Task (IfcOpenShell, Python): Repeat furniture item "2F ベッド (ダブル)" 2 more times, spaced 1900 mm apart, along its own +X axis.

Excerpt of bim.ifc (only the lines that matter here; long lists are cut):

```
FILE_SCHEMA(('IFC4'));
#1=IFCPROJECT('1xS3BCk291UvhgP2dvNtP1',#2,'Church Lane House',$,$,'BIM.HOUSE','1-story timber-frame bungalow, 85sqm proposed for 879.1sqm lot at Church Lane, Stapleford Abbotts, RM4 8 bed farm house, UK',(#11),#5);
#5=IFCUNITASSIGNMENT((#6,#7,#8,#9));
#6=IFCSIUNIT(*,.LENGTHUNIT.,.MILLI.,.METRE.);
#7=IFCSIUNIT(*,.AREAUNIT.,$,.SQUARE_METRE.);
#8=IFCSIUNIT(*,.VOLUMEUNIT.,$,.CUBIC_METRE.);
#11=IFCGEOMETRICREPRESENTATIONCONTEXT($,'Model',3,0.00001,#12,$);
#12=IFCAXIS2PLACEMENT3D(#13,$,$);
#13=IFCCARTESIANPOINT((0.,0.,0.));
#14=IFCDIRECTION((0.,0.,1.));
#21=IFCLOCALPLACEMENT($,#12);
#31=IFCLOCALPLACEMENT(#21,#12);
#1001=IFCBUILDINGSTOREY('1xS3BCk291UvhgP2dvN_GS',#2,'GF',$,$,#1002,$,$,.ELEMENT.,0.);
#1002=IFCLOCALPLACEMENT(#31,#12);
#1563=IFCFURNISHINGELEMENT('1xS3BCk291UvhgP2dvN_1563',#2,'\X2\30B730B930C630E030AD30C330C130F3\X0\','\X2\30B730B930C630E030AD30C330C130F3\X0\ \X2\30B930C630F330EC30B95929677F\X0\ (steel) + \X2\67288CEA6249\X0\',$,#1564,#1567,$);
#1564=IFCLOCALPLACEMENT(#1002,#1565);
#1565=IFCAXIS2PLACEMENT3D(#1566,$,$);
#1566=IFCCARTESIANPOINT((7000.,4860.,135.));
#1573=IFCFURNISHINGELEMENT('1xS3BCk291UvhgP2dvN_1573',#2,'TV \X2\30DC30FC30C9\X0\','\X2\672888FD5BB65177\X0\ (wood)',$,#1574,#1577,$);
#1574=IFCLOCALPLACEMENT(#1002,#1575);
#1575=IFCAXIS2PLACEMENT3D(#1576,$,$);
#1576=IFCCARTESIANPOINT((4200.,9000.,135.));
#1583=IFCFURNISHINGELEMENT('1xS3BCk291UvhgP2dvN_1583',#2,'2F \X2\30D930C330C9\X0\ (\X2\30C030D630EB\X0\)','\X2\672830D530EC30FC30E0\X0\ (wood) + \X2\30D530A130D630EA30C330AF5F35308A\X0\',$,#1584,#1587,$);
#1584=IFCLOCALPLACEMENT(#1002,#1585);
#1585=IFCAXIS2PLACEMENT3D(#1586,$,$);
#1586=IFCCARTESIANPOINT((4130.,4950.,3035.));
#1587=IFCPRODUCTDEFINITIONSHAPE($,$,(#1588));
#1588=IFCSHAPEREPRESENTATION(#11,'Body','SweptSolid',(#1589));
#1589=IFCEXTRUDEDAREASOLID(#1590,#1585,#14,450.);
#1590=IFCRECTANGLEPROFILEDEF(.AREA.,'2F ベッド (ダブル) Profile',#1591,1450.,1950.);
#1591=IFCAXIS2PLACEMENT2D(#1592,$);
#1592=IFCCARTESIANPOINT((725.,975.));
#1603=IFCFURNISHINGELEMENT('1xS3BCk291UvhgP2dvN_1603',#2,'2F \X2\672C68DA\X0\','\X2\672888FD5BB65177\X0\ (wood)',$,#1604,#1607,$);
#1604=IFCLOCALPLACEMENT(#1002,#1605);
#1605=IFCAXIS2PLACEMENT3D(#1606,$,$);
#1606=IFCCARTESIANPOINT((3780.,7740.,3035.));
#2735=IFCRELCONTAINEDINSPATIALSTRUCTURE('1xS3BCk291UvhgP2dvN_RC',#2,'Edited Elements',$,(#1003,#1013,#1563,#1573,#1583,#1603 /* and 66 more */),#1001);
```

```python
import ifcopenshell
import ifcopenshell.api.geometry
import ifcopenshell.api.root
import ifcopenshell.util.element
import ifcopenshell.util.placement

model = ifcopenshell.open("bim.ifc")


def reuse_history(source, copy):
    """copy_class also copies each property set's owner history, people and application; keep the originals."""
    for rel in copy.IsDefinedBy:
        if rel.is_a("IfcRelDefinesByProperties") and (history := rel.RelatingPropertyDefinition.OwnerHistory):
            rel.RelatingPropertyDefinition.OwnerHistory = source.OwnerHistory
            ifcopenshell.util.element.remove_deep2(model, history)


source = model.by_guid("1xS3BCk291UvhgP2dvN_1583")
base = ifcopenshell.util.placement.get_local_placement(source.ObjectPlacement)
step = base[:3, 0] * 1900.0

for i in range(1, 3):
    copy = ifcopenshell.api.root.copy_class(model, product=source)
    copy.Representation = ifcopenshell.util.element.copy_deep(
        model, source.Representation, exclude=["IfcGeometricRepresentationContext", "IfcRepresentationMap"]
    )
    reuse_history(source, copy)
    matrix = base.copy()
    matrix[:3, 3] += i * step
    print("added at", matrix[:3, 3].round(3) + 0.0)
    ifcopenshell.api.geometry.edit_object_placement(model, product=copy, matrix=matrix, is_si=False)

model.write("bim_rev.ifc")
```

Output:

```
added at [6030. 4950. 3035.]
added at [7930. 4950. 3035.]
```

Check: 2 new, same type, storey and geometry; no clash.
